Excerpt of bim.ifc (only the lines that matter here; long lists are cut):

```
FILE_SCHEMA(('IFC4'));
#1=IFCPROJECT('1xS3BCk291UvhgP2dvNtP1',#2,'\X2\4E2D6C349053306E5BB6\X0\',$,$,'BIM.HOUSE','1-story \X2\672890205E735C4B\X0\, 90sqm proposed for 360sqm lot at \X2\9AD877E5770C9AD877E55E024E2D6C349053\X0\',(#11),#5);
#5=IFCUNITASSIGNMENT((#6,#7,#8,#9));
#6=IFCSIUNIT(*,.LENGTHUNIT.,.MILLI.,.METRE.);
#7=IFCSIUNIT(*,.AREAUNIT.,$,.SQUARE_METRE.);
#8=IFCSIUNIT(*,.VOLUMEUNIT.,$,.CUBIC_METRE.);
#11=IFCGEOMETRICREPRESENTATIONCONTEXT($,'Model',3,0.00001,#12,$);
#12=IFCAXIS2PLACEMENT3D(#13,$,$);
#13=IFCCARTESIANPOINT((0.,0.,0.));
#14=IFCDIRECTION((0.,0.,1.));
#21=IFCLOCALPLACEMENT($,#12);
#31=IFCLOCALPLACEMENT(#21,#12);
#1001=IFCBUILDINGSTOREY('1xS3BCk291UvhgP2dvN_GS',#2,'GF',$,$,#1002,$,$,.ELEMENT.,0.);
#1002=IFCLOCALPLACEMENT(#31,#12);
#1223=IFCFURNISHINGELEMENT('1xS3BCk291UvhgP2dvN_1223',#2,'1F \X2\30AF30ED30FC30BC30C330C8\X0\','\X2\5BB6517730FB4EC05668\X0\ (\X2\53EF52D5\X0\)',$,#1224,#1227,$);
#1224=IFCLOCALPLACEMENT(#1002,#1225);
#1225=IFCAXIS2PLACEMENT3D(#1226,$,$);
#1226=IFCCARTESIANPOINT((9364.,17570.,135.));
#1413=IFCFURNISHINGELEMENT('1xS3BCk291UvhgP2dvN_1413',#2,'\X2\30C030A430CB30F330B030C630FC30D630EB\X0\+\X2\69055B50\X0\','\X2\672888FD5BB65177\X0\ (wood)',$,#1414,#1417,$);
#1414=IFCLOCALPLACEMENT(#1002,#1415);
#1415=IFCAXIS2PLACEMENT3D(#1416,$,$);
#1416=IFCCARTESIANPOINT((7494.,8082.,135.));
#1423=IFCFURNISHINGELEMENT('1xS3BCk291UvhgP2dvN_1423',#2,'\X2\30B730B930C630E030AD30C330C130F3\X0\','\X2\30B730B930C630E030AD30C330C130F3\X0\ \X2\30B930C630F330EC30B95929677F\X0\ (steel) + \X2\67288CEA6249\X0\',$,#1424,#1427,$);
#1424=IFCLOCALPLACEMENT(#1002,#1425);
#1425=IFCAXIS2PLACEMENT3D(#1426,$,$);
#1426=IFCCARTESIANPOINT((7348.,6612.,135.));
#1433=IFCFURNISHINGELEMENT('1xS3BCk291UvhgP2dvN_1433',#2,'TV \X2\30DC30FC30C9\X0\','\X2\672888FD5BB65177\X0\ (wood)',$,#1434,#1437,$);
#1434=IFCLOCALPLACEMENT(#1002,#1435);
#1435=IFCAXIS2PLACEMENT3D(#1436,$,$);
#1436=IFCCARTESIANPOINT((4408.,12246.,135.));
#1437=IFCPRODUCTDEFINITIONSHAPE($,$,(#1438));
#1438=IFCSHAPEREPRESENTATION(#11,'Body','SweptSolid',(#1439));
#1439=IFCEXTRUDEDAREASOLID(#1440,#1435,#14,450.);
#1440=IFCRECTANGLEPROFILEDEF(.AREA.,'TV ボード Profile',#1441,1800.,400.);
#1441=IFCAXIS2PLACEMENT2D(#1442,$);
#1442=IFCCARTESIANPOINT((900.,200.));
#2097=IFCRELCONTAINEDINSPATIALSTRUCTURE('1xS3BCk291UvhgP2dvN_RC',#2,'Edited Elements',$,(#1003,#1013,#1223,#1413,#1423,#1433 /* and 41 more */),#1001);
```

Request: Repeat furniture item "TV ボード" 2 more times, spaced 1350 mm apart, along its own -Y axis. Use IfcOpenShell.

```python
import ifcopenshell
import ifcopenshell.api.geometry
import ifcopenshell.api.root
import ifcopenshell.util.element
import ifcopenshell.util.placement
import ifcopenshell.util.unit

model = ifcopenshell.open("bim.ifc")
unit_scale = ifcopenshell.util.unit.calculate_unit_scale(model)


def reuse_history(source, copy):
    """copy_class also copies each property set's owner history, people and application; keep the originals."""
    for rel in copy.IsDefinedBy:
        if rel.is_a("IfcRelDefinesByProperties") and (history := rel.RelatingPropertyDefinition.OwnerHistory):
            rel.RelatingPropertyDefinition.OwnerHistory = source.OwnerHistory
            ifcopenshell.util.element.remove_deep2(model, history)


source = model.by_guid("1xS3BCk291UvhgP2dvN_1433")
base = ifcopenshell.util.placement.get_local_placement(source.ObjectPlacement)
step = -base[:3, 1] * 1.35 / unit_scale

for i in range(1, 3):
    copy = ifcopenshell.api.root.copy_class(model, product=source)
    copy.Representation = ifcopenshell.util.element.copy_deep(
        model, source.Representation, exclude=["IfcGeometricRepresentationContext", "IfcRepresentationMap"]
    )
    reuse_history(source, copy)
    matrix = base.copy()
    matrix[:3, 3] += i * step
    print("added at", matrix[:3, 3].round(3) + 0.0)
    ifcopenshell.api.geometry.edit_object_placement(model, product=copy, matrix=matrix, is_si=False)

model.write("bim_rev.ifc")
```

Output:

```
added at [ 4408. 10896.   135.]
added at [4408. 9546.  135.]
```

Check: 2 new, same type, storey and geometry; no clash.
